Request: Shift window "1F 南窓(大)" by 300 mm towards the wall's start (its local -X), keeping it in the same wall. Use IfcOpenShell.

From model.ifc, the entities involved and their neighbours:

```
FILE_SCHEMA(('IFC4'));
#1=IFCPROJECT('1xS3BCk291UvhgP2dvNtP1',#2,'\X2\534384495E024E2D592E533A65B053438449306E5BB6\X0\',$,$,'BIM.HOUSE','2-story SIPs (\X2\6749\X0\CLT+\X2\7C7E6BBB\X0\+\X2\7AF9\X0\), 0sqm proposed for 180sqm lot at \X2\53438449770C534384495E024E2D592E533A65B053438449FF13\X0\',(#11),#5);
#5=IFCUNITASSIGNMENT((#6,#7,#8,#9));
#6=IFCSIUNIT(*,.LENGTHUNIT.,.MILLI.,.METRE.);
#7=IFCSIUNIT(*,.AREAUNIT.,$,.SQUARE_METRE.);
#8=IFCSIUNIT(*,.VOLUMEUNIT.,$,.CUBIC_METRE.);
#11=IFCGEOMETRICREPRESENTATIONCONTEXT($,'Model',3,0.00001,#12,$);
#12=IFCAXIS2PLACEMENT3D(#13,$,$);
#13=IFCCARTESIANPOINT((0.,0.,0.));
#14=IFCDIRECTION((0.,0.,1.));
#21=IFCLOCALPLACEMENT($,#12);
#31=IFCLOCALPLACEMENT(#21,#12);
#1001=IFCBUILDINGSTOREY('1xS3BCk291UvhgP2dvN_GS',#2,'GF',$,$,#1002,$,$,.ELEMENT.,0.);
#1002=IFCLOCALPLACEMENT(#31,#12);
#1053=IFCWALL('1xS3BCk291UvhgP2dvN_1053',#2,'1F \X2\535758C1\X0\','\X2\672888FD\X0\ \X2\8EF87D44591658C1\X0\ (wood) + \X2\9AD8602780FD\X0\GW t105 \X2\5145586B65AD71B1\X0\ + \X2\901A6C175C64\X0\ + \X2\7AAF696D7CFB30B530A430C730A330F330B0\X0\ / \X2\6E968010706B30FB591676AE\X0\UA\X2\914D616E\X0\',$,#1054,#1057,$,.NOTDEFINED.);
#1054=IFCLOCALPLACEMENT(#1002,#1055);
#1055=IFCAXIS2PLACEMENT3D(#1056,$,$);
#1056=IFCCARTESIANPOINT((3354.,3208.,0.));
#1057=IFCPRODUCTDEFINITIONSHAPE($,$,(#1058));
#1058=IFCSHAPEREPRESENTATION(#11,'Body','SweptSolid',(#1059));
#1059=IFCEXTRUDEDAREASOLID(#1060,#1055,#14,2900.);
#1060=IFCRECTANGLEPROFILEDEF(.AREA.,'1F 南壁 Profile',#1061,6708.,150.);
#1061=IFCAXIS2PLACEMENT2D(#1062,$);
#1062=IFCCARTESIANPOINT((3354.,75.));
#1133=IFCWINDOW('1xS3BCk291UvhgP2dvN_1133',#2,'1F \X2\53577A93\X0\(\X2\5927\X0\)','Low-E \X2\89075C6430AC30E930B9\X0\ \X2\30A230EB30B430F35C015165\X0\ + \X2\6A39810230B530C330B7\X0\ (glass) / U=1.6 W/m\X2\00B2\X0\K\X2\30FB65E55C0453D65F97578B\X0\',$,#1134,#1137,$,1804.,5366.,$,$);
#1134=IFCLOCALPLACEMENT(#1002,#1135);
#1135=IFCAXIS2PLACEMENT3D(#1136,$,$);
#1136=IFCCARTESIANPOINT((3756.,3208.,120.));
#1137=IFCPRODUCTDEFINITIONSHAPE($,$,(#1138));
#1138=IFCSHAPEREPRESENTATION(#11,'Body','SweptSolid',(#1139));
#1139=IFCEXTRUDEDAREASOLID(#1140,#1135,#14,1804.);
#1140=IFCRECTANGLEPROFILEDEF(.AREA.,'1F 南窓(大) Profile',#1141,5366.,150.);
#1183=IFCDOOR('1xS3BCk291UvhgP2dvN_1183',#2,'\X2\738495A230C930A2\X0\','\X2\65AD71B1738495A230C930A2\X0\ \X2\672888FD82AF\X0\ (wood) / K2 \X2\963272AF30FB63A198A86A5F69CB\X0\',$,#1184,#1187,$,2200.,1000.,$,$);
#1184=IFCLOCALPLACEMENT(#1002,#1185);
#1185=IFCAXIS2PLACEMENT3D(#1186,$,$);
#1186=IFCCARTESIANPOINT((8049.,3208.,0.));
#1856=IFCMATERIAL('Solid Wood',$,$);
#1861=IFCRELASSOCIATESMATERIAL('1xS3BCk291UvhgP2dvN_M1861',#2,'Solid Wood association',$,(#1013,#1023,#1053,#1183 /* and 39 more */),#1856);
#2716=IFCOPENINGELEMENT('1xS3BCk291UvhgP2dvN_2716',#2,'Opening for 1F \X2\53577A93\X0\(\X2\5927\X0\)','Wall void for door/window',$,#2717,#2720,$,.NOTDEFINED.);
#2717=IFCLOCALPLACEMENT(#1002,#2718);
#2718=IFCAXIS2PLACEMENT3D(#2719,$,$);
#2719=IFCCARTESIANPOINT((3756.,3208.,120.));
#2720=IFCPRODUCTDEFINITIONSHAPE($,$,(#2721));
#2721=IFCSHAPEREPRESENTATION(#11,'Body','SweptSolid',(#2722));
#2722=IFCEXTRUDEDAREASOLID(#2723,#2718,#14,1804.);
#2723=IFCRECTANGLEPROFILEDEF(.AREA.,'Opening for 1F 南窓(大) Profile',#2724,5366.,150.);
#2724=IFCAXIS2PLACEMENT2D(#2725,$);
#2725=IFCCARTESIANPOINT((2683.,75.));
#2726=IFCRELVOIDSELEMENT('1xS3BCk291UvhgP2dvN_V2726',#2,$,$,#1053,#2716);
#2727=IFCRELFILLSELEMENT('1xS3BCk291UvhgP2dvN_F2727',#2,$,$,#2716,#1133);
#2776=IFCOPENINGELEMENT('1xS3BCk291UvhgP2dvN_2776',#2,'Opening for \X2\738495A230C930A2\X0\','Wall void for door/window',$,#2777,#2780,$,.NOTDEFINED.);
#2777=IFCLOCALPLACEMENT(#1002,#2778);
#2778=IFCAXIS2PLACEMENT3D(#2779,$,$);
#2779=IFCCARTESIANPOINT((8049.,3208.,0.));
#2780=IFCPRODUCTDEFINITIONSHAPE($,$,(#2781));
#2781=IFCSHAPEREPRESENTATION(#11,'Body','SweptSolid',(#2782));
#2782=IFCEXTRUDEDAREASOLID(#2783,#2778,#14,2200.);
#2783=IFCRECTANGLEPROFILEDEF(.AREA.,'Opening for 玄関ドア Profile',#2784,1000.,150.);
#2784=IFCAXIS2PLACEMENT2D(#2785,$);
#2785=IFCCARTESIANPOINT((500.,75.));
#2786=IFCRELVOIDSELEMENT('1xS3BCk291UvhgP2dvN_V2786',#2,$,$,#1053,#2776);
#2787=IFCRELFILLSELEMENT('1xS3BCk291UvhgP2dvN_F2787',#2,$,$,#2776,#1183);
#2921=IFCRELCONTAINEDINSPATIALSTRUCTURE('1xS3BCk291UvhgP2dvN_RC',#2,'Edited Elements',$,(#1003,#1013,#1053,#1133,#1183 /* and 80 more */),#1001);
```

```python
import ifcopenshell
import ifcopenshell.api.geometry
import ifcopenshell.util.placement
import ifcopenshell.util.unit

model = ifcopenshell.open("model.ifc")
unit_scale = ifcopenshell.util.unit.calculate_unit_scale(model)

window = model.by_guid("1xS3BCk291UvhgP2dvN_1133")
opening = window.FillsVoids[0].RelatingOpeningElement
wall = opening.VoidsElements[0].RelatingBuildingElement

wall_matrix = ifcopenshell.util.placement.get_local_placement(wall.ObjectPlacement)
shift = wall_matrix[:3, 0] * -0.3 / unit_scale
before = ifcopenshell.util.placement.get_local_placement(window.ObjectPlacement)[:3, 3].copy()

# The window is not placed relative to its opening, so move both.
for product in (opening, window):
    matrix = ifcopenshell.util.placement.get_local_placement(product.ObjectPlacement)
    matrix[:3, 3] += shift
    ifcopenshell.api.geometry.edit_object_placement(model, product=product, matrix=matrix, is_si=False)

after = ifcopenshell.util.placement.get_local_placement(window.ObjectPlacement)[:3, 3]
print("window moved by", (after - before).round(3) + 0.0)

model.write("model_edited.ifc")
```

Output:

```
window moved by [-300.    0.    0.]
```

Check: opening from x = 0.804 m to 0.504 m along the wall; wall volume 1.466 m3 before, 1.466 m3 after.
